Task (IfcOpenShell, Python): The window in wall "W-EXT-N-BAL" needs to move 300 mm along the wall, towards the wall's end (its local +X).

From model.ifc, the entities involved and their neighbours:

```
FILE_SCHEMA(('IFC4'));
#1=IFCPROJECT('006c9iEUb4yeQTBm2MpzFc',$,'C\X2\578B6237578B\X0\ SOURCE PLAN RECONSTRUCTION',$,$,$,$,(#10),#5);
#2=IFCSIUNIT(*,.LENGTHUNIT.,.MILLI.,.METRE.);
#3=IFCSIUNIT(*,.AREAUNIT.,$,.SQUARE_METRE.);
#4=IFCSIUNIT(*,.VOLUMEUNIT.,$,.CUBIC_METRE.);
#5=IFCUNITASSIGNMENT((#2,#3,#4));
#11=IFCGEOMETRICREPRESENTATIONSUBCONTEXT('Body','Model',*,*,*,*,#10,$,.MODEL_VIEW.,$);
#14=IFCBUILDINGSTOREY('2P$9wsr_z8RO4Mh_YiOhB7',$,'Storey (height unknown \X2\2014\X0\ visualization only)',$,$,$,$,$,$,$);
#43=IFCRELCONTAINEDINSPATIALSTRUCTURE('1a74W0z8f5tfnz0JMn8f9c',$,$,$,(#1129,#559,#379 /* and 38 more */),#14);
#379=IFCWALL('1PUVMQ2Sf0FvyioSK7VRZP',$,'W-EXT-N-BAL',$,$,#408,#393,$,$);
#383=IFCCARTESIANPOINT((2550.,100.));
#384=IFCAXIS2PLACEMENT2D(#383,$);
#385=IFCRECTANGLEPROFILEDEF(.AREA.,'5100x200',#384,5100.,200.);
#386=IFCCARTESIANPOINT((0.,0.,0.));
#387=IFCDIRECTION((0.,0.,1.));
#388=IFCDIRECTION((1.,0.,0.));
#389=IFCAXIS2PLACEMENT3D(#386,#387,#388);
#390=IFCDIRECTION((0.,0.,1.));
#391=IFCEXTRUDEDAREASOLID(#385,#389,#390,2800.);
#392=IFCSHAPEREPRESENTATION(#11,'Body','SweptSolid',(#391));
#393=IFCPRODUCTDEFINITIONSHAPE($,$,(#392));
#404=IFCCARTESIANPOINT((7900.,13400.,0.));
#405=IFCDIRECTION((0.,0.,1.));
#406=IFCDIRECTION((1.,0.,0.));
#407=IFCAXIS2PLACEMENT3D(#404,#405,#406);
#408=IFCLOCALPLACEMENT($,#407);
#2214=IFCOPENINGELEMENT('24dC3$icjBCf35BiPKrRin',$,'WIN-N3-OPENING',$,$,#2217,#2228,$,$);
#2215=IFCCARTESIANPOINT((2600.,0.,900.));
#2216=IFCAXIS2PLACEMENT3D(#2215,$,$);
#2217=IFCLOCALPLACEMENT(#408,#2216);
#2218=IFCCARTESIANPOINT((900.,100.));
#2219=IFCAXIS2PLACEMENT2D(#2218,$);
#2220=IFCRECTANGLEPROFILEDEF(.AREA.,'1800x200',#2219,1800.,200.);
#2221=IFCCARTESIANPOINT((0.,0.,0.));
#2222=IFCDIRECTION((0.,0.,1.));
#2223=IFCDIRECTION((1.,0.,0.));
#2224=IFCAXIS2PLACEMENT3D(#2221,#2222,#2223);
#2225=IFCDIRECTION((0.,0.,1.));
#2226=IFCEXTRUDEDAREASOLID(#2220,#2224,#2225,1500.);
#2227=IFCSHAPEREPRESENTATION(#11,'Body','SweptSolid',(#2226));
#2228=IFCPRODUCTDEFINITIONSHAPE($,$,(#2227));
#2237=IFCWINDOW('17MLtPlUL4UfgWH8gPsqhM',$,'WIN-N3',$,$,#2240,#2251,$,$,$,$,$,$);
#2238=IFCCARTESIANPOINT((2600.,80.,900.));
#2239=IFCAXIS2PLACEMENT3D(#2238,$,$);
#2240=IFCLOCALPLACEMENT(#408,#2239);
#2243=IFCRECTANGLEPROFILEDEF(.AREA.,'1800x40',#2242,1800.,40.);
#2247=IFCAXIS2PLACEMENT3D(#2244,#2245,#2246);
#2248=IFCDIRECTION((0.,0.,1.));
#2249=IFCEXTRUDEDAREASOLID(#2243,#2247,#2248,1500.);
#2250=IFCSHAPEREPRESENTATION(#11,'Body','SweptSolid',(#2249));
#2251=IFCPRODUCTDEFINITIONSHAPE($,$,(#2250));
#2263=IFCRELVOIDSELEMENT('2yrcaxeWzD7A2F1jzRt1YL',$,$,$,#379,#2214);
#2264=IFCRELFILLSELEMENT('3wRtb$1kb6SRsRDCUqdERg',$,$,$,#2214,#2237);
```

```python
import ifcopenshell
import ifcopenshell.api.geometry
import ifcopenshell.util.placement
import ifcopenshell.util.unit

model = ifcopenshell.open("model.ifc")
unit_scale = ifcopenshell.util.unit.calculate_unit_scale(model)

window = model.by_id(2237)
opening = window.FillsVoids[0].RelatingOpeningElement
wall = opening.VoidsElements[0].RelatingBuildingElement

wall_matrix = ifcopenshell.util.placement.get_local_placement(wall.ObjectPlacement)
shift = wall_matrix[:3, 0] * 0.3 / unit_scale
before = ifcopenshell.util.placement.get_local_placement(window.ObjectPlacement)[:3, 3].copy()

# The window is not placed relative to its opening, so move both.
for product in (opening, window):
    matrix = ifcopenshell.util.placement.get_local_placement(product.ObjectPlacement)
    matrix[:3, 3] += shift
    ifcopenshell.api.geometry.edit_object_placement(model, product=product, matrix=matrix, is_si=False)

after = ifcopenshell.util.placement.get_local_placement(window.ObjectPlacement)[:3, 3]
print("window moved by", (after - before).round(3) + 0.0)

model.write("model_v2.ifc")
```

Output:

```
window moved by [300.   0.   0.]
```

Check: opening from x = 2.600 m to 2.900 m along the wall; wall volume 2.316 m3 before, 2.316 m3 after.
